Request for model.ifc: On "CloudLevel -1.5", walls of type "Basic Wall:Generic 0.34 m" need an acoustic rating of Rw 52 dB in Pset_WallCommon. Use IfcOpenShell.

First a look at what the model holds.

```python
import ifcopenshell
import ifcopenshell.util.element

model = ifcopenshell.open("model.ifc")
print(model.schema)
storey = next(s for s in model.by_type("IfcBuildingStorey") if s.Name == "CloudLevel -1.5")
walls = [e for e in ifcopenshell.util.element.get_decomposition(storey) if e.is_a("IfcWall")]
seen = {}
for e in walls:
    element_type = ifcopenshell.util.element.get_type(e)
    key = (element_type.Name if element_type != e and element_type else None, ifcopenshell.util.element.get_pset(e, "Pset_WallCommon", "AcousticRating"))
    seen[key] = seen.get(key, 0) + 1
for (name, value), count in sorted(seen.items(), key=str):
    print(count, "x", name, "|", value)
```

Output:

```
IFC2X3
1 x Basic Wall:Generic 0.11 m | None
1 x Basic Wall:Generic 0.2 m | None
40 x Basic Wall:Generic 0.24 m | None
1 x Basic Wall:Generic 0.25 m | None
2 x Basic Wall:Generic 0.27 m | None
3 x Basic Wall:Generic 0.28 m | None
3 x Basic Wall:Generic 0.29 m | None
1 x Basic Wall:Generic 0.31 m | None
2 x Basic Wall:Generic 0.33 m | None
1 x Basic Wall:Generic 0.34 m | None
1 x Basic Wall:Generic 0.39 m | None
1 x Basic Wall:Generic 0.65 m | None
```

```python
import ifcopenshell
import ifcopenshell.api.pset
import ifcopenshell.util.element

model = ifcopenshell.open("model.ifc")

storey = next(s for s in model.by_type("IfcBuildingStorey") if s.Name == "CloudLevel -1.5")
walls = [e for e in ifcopenshell.util.element.get_decomposition(storey) if e.is_a("IfcWall")]

count = 0
for e in walls:
    element_type = ifcopenshell.util.element.get_type(e)
    if element_type in (None, e) or element_type.Name != "Basic Wall:Generic 0.34 m":
        continue
    # add_pset returns the element's existing set when there is one.
    pset = ifcopenshell.api.pset.add_pset(model, product=e, name="Pset_WallCommon")
    ifcopenshell.api.pset.edit_pset(model, pset=pset, properties={"AcousticRating": "Rw 52 dB"})
    count += 1

print(count, "walls updated")

model.write("model_rev.ifc")
```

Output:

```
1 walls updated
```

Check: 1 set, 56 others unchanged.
